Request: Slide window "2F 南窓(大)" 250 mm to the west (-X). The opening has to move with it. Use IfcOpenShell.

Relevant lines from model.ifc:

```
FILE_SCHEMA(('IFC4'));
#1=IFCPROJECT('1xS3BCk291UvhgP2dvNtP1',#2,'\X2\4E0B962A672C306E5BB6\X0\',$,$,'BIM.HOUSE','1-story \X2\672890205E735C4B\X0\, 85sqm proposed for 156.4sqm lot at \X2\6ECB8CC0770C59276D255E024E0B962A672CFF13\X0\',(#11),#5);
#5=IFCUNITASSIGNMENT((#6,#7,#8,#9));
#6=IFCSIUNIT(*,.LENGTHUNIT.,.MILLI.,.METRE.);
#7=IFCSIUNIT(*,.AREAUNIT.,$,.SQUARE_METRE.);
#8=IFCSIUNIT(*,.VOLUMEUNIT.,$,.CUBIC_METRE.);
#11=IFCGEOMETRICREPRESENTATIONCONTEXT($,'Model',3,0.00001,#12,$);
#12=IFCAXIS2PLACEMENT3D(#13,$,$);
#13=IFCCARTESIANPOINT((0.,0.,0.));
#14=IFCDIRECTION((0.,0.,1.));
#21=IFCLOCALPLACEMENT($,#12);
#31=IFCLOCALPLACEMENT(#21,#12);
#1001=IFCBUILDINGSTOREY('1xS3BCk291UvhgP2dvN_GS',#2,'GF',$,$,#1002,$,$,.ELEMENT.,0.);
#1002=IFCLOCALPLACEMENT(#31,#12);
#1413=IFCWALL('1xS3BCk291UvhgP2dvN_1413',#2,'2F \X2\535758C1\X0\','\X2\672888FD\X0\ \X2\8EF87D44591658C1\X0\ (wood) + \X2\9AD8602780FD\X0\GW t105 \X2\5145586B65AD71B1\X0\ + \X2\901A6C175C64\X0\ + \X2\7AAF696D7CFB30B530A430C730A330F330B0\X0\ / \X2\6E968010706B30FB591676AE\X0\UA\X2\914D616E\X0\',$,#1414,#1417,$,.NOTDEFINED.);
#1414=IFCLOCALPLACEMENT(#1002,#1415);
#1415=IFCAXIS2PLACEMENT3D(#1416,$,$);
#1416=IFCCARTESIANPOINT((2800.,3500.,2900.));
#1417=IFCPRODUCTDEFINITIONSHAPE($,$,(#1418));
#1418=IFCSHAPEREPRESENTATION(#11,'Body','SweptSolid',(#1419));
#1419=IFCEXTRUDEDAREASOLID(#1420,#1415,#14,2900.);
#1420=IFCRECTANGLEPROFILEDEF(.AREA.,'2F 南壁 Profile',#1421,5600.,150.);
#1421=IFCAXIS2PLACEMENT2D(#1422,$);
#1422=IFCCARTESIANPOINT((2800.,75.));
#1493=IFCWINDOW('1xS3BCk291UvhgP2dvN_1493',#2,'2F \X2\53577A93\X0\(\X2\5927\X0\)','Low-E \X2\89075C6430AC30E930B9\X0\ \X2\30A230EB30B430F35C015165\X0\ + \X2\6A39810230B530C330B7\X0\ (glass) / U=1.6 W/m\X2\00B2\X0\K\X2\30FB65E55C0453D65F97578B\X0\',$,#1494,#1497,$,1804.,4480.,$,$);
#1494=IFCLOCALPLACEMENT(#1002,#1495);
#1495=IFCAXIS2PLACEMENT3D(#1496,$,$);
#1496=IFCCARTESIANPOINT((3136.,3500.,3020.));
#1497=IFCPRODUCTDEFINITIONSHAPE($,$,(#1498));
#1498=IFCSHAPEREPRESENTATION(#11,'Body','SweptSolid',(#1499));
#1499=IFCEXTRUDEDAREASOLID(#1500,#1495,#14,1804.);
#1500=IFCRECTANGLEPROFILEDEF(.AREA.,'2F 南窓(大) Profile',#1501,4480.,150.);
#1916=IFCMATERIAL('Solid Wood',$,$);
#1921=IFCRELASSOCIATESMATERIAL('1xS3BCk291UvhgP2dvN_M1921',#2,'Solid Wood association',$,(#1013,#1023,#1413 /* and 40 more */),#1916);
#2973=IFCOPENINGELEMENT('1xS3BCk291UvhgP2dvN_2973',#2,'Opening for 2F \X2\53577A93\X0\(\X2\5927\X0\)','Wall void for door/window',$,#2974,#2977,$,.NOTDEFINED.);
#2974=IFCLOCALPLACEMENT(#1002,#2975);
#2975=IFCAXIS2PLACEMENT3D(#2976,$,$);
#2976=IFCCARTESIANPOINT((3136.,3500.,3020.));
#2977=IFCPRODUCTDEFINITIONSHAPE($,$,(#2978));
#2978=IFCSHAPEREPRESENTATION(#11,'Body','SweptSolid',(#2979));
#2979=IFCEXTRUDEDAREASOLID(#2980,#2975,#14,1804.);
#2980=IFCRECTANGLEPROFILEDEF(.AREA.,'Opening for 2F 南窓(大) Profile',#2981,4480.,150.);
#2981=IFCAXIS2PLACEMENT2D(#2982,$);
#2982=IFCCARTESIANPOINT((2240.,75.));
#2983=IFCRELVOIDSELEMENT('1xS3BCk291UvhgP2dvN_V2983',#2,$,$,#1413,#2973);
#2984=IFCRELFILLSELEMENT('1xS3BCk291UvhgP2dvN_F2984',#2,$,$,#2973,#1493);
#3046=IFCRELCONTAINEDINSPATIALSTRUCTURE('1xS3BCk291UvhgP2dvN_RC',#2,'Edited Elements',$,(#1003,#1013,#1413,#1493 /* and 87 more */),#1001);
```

```python
import ifcopenshell
import ifcopenshell.api.geometry
import ifcopenshell.util.placement
import ifcopenshell.util.unit

model = ifcopenshell.open("model.ifc")
unit_scale = ifcopenshell.util.unit.calculate_unit_scale(model)

window = model.by_guid("1xS3BCk291UvhgP2dvN_1493")
opening = window.FillsVoids[0].RelatingOpeningElement
wall = opening.VoidsElements[0].RelatingBuildingElement

wall_matrix = ifcopenshell.util.placement.get_local_placement(wall.ObjectPlacement)
shift = wall_matrix[:3, 0] * -0.25 / unit_scale
before = ifcopenshell.util.placement.get_local_placement(window.ObjectPlacement)[:3, 3].copy()

# The window is not placed relative to its opening, so move both.
for product in (opening, window):
    matrix = ifcopenshell.util.placement.get_local_placement(product.ObjectPlacement)
    matrix[:3, 3] += shift
    ifcopenshell.api.geometry.edit_object_placement(model, product=product, matrix=matrix, is_si=False)

after = ifcopenshell.util.placement.get_local_placement(window.ObjectPlacement)[:3, 3]
print("window moved by", (after - before).round(3) + 0.0)

model.write("model-out.ifc")
```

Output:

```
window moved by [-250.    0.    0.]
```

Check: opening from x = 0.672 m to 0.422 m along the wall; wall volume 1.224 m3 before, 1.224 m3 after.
